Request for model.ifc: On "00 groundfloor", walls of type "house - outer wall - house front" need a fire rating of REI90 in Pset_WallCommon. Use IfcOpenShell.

First a look at what the model holds.

```python
import ifcopenshell
import ifcopenshell.util.element

model = ifcopenshell.open("model.ifc")
print(model.schema)
storey = next(s for s in model.by_type("IfcBuildingStorey") if s.Name == "00 groundfloor")
walls = [e for e in ifcopenshell.util.element.get_decomposition(storey) if e.is_a("IfcWall")]
seen = {}
for e in walls:
    element_type = ifcopenshell.util.element.get_type(e)
    key = (element_type.Name if element_type != e and element_type else None, ifcopenshell.util.element.get_pset(e, "Pset_WallCommon", "FireRating"))
    seen[key] = seen.get(key, 0) + 1
for (name, value), count in sorted(seen.items(), key=str):
    print(count, "x", name, "|", value)
```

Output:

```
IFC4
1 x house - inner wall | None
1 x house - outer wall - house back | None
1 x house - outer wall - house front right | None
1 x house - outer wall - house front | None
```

```python
import ifcopenshell
import ifcopenshell.api.pset
import ifcopenshell.util.element

model = ifcopenshell.open("model.ifc")

storey = next(s for s in model.by_type("IfcBuildingStorey") if s.Name == "00 groundfloor")
walls = [e for e in ifcopenshell.util.element.get_decomposition(storey) if e.is_a("IfcWall")]

count = 0
for e in walls:
    element_type = ifcopenshell.util.element.get_type(e)
    if element_type in (None, e) or element_type.Name != "house - outer wall - house front":
        continue
    # add_pset returns the element's existing set when there is one.
    pset = ifcopenshell.api.pset.add_pset(model, product=e, name="Pset_WallCommon")
    ifcopenshell.api.pset.edit_pset(model, pset=pset, properties={"FireRating": "REI90"})
    count += 1

print(count, "walls updated")

model.write("model_v2.ifc")
```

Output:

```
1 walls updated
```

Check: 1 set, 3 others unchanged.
